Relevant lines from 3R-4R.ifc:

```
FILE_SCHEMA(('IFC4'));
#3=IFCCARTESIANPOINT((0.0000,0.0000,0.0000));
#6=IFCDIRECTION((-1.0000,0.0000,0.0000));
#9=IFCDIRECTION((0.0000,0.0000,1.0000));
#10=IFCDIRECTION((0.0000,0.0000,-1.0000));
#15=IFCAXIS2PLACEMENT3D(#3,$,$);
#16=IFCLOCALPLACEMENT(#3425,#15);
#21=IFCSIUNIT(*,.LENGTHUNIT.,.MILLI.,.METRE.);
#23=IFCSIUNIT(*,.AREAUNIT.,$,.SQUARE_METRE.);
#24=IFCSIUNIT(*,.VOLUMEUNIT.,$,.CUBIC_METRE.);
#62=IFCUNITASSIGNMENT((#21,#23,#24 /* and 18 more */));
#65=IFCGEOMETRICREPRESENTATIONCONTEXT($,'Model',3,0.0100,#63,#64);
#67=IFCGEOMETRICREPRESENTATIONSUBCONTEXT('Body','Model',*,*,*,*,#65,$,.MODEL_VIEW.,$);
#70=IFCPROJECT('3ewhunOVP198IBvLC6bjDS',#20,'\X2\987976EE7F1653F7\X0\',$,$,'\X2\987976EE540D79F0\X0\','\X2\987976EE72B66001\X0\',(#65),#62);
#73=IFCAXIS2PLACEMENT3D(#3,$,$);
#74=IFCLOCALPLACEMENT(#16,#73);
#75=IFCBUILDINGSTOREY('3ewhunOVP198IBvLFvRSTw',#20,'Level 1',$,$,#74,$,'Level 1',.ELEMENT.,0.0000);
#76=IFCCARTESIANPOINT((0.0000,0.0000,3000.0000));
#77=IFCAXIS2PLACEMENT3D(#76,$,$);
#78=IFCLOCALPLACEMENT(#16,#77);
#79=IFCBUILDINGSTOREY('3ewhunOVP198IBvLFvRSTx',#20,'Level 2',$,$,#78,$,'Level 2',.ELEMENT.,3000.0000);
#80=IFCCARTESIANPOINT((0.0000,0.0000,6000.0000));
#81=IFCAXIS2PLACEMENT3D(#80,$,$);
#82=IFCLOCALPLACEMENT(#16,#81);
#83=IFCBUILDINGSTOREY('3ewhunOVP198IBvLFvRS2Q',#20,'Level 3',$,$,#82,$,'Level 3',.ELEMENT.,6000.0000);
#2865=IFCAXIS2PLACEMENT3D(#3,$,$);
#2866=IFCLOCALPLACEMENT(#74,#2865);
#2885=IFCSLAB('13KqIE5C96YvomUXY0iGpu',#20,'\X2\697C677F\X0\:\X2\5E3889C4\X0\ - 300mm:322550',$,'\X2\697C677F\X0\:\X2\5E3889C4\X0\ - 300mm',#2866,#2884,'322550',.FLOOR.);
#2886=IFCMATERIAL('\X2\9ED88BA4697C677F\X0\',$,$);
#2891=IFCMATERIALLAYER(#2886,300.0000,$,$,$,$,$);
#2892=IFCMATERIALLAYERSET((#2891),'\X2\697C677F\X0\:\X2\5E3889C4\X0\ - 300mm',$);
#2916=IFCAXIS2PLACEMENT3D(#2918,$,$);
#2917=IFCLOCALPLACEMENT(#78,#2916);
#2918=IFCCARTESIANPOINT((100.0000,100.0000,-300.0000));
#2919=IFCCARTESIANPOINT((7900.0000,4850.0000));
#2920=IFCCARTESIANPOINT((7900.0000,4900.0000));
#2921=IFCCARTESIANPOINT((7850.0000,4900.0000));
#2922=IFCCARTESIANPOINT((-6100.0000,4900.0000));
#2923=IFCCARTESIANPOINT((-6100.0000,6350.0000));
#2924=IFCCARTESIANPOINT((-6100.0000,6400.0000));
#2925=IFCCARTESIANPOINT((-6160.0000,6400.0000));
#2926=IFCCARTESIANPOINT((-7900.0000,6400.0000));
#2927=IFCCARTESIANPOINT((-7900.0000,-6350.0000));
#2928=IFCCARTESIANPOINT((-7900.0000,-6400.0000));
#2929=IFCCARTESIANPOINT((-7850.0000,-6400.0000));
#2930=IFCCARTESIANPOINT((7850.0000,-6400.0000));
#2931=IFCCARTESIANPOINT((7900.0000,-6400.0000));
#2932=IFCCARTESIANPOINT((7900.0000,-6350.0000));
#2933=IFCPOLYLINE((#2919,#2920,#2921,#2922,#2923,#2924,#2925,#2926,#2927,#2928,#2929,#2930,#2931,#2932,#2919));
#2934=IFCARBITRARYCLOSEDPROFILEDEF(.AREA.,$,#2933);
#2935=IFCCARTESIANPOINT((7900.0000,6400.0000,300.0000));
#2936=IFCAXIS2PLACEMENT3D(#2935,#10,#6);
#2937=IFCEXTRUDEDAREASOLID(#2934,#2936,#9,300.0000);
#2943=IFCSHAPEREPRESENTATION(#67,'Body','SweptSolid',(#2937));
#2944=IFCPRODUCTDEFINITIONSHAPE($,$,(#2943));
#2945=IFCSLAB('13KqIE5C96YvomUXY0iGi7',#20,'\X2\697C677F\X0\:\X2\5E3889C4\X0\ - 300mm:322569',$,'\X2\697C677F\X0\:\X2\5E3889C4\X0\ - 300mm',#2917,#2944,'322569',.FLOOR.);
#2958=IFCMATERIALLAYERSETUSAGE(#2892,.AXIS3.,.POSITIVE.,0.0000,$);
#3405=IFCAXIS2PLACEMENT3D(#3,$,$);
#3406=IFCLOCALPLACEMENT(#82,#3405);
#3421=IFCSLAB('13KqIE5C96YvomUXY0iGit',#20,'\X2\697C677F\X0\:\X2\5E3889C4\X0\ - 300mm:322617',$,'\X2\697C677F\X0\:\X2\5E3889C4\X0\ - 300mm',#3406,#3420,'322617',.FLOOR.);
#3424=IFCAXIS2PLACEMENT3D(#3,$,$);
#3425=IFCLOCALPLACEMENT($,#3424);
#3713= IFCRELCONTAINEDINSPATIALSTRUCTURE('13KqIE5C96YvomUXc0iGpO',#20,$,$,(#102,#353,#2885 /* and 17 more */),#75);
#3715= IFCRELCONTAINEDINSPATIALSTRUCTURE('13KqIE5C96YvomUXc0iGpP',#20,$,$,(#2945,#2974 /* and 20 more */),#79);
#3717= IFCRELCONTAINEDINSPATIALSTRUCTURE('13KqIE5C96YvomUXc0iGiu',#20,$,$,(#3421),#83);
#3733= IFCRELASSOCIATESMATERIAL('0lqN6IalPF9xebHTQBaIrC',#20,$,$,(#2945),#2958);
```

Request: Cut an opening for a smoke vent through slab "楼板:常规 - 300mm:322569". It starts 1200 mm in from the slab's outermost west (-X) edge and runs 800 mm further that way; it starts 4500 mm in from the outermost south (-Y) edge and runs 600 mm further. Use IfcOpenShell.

```python
import numpy as np
import ifcopenshell
import ifcopenshell.api.feature
import ifcopenshell.api.geometry
import ifcopenshell.api.root
import ifcopenshell.geom
import ifcopenshell.util.placement
import ifcopenshell.util.representation
import ifcopenshell.util.shape
import ifcopenshell.util.unit

model = ifcopenshell.open("3R-4R.ifc")
unit_scale = ifcopenshell.util.unit.calculate_unit_scale(model)
settings = ifcopenshell.geom.settings()


def volume(element):
    """Net volume in cubic metres, openings subtracted."""
    shape = ifcopenshell.geom.create_shape(settings, element)
    return ifcopenshell.util.shape.get_volume(shape.geometry)


slab = model.by_id(2945)
before = volume(slab)

# Extent in the slab's own axes, in metres. The edges named are its -X and -Y sides.
slab_shape = ifcopenshell.geom.create_shape(settings, slab)
vertices = ifcopenshell.util.shape.get_vertices(slab_shape.geometry)
x_min, y_min, bottom = vertices.min(axis=0)
top = vertices[:, 2].max()

opening = ifcopenshell.api.root.create_entity(model, ifc_class="IfcOpeningElement", name="Smoke vent opening", predefined_type="OPENING")
context = ifcopenshell.util.representation.get_context(model, "Model", "Body", "MODEL_VIEW")
width, depth = 0.8, 0.6
outline = [(0.0, 0.0), (width, 0.0), (width, depth), (0.0, depth), (0.0, 0.0)]
# Overshoot both faces by 50 mm so the cut is clean.
shape = ifcopenshell.api.geometry.add_slab_representation(
    model, context=context, depth=top - bottom + 0.1, polyline=outline
)
ifcopenshell.api.geometry.assign_representation(model, product=opening, representation=shape)

matrix = ifcopenshell.util.placement.get_local_placement(slab.ObjectPlacement)
matrix[:, 3] = matrix @ np.append(np.array([x_min + 1.2, y_min + 4.5, bottom - 0.05]) / unit_scale, 1.0)
ifcopenshell.api.geometry.edit_object_placement(model, product=opening, matrix=matrix, is_si=False)
ifcopenshell.api.feature.add_feature(model, feature=opening, element=slab)

after = volume(slab)

print(f"slab volume {before:.3f} -> {after:.3f} m3")

model.write("3R-4R_rev.ifc")
```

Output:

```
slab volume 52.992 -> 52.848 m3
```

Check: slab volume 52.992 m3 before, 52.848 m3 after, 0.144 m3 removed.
